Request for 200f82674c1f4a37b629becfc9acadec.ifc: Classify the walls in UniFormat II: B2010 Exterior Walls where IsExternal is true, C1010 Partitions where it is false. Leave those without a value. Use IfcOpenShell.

First a look at what the model holds.

```python
import ifcopenshell
import ifcopenshell.util.element

model = ifcopenshell.open("200f82674c1f4a37b629becfc9acadec.ifc")
print(model.schema)
print("classifications:", [c.Name for c in model.by_type("IfcClassification")])
values = [ifcopenshell.util.element.get_pset(e, "Pset_WallCommon", "IsExternal") for e in model.by_type("IfcWall")]
for value in (True, False, None):
    print("IsExternal", value, values.count(value))
```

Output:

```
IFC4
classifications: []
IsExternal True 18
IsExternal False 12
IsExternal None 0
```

```python
import ifcopenshell
import ifcopenshell.api.classification
import ifcopenshell.util.element

model = ifcopenshell.open("200f82674c1f4a37b629becfc9acadec.ifc")

system = ifcopenshell.api.classification.add_classification(model, classification="UniFormat II")

walls = model.by_type("IfcWall")
external = {e: ifcopenshell.util.element.get_pset(e, "Pset_WallCommon", "IsExternal") for e in walls}
for flag, code, name in ((True, "B2010", "Exterior Walls"), (False, "C1010", "Partitions")):
    products = [e for e in walls if external[e] is flag]
    ifcopenshell.api.classification.add_reference(
        model, products=products, classification=system, identification=code, name=name
    )
    print(code, len(products))

model.write("200f82674c1f4a37b629becfc9acadec_edited.ifc")
```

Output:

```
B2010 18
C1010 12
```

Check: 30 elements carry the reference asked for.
